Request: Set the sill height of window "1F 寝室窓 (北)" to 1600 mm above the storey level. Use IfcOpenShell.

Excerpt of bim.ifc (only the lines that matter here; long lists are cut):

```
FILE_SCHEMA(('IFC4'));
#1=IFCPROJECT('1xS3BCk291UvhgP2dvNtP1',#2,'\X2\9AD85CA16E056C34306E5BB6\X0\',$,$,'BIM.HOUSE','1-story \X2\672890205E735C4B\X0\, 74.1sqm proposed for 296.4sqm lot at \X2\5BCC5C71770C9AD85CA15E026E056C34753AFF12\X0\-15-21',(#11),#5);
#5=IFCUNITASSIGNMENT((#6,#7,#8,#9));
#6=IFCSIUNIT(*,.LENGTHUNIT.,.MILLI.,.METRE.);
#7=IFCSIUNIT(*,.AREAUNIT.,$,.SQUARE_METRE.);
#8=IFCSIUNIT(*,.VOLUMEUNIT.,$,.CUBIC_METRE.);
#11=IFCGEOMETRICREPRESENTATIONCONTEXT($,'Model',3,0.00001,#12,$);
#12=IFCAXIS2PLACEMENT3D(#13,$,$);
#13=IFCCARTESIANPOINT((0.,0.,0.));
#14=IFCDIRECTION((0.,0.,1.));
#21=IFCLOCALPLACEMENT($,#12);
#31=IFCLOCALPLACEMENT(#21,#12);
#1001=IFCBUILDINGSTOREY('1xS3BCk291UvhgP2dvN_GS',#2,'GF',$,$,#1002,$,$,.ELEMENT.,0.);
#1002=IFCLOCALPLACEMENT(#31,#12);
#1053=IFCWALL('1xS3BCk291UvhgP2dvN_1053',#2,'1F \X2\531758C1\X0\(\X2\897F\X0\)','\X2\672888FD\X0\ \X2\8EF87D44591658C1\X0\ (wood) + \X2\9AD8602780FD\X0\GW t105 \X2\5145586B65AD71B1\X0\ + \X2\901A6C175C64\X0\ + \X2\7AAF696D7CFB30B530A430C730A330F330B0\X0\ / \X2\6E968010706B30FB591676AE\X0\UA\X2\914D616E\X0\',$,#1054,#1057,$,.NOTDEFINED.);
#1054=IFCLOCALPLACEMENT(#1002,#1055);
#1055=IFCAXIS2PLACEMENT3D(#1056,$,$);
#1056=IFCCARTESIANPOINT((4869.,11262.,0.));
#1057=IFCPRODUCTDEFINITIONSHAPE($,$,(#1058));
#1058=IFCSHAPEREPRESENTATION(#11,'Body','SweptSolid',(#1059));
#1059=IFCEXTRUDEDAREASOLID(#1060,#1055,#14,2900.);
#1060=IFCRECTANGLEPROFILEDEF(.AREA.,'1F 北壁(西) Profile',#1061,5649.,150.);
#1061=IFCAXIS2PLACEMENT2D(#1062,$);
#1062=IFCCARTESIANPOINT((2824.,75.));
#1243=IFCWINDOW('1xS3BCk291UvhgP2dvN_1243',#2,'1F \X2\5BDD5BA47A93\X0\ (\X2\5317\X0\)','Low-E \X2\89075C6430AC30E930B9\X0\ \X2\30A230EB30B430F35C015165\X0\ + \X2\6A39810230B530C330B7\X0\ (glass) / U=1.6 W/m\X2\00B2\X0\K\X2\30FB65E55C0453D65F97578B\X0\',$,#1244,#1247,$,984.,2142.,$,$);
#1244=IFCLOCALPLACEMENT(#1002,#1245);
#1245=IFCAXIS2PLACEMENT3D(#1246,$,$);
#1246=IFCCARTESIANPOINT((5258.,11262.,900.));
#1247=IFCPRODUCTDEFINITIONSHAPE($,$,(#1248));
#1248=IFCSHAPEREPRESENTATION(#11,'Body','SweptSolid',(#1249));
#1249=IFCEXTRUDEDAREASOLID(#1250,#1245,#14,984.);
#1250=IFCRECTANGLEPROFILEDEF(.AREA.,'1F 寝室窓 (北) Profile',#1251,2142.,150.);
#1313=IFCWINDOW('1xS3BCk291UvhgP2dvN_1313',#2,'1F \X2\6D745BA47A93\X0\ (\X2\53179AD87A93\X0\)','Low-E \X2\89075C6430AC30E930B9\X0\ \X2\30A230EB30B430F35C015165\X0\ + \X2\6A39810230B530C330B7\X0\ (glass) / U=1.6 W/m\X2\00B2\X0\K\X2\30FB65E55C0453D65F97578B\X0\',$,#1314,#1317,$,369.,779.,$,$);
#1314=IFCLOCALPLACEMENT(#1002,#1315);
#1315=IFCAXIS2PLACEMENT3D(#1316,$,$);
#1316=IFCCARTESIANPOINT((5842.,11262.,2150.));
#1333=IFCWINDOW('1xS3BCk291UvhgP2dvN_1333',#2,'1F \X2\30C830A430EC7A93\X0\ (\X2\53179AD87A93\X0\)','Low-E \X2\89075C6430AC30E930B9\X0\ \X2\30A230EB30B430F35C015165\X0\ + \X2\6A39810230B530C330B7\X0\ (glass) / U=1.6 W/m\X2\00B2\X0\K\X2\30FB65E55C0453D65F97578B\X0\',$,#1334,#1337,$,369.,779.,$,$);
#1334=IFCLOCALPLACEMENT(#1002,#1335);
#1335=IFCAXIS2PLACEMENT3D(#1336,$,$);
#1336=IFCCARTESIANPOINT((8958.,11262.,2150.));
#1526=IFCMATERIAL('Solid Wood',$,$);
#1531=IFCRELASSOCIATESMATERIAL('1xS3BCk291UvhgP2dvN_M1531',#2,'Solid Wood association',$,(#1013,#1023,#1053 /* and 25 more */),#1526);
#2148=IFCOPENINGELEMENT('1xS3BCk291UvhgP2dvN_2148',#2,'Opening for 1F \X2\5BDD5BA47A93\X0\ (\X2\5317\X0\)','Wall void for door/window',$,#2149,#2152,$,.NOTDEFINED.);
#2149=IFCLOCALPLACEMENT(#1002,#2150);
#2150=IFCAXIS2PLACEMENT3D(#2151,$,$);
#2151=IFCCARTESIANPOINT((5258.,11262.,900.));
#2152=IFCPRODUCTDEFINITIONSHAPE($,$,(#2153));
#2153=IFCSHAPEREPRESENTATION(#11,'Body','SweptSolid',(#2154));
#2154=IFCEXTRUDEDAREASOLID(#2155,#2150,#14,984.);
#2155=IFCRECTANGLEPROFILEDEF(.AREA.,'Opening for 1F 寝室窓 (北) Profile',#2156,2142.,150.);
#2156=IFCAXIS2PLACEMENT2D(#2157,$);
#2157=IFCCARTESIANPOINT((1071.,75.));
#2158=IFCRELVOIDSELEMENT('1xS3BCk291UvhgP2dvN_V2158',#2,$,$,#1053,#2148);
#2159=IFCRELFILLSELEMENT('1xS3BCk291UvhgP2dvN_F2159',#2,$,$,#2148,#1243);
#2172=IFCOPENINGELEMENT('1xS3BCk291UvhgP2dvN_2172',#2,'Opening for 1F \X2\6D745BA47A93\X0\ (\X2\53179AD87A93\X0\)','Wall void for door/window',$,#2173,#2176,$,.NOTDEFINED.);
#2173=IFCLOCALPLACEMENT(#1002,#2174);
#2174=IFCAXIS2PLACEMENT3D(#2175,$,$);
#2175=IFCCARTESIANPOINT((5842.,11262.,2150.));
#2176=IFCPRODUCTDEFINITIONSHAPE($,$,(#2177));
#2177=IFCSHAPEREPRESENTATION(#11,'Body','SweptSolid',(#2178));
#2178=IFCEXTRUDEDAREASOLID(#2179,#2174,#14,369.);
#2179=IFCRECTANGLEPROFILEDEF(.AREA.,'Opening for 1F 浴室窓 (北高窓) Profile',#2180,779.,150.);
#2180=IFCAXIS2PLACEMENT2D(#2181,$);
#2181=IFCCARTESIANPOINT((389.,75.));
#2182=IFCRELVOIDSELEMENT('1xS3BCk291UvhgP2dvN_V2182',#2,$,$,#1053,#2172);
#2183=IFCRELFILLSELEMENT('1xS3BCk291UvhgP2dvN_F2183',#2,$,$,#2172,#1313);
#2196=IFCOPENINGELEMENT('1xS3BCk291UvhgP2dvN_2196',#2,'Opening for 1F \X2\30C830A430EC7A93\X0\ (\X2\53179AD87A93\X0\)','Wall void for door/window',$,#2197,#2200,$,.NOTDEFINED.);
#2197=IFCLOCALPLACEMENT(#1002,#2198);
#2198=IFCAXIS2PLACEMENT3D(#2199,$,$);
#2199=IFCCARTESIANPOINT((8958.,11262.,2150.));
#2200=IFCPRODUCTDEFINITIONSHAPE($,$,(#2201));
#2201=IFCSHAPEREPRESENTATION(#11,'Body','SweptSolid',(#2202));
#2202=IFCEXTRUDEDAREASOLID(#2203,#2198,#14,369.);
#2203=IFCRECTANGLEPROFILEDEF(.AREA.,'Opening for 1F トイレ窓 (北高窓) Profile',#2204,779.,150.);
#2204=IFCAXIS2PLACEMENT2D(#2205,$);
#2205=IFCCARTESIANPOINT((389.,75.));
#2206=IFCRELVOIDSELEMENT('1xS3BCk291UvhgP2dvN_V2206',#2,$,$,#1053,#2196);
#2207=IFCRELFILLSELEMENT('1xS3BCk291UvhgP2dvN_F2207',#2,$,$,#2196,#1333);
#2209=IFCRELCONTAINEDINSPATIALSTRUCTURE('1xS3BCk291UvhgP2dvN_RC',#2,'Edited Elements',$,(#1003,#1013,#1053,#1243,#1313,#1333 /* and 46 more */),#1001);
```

```python
import numpy as np
import ifcopenshell
import ifcopenshell.api.geometry
import ifcopenshell.geom
import ifcopenshell.util.element
import ifcopenshell.util.placement
import ifcopenshell.util.shape
import ifcopenshell.util.unit

model = ifcopenshell.open("bim.ifc")
unit_scale = ifcopenshell.util.unit.calculate_unit_scale(model)

window = model.by_guid("1xS3BCk291UvhgP2dvN_1243")
opening = window.FillsVoids[0].RelatingOpeningElement
storey = ifcopenshell.util.element.get_container(window, ifc_class="IfcBuildingStorey")
level = ifcopenshell.util.placement.get_local_placement(storey.ObjectPlacement)[2, 3]

# The opening's origin need not be at the sill, so measure its lowest point.
shape = ifcopenshell.geom.create_shape(ifcopenshell.geom.settings(), opening)
bottom = ifcopenshell.util.shape.get_shape_bottom_elevation(shape, shape.geometry) / unit_scale
dz = level + 1600.0 - bottom

shift = np.array([0.0, 0.0, dz])
# The window is not placed relative to its opening, so move both.
for product in (opening, window):
    matrix = ifcopenshell.util.placement.get_local_placement(product.ObjectPlacement)
    matrix[:3, 3] += shift
    ifcopenshell.api.geometry.edit_object_placement(model, product=product, matrix=matrix, is_si=False)

print(f"moved by {dz * unit_scale:+.3f} m")

model.write("bim_rev.ifc")
```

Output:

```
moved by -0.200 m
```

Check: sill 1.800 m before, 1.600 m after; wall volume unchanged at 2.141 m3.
